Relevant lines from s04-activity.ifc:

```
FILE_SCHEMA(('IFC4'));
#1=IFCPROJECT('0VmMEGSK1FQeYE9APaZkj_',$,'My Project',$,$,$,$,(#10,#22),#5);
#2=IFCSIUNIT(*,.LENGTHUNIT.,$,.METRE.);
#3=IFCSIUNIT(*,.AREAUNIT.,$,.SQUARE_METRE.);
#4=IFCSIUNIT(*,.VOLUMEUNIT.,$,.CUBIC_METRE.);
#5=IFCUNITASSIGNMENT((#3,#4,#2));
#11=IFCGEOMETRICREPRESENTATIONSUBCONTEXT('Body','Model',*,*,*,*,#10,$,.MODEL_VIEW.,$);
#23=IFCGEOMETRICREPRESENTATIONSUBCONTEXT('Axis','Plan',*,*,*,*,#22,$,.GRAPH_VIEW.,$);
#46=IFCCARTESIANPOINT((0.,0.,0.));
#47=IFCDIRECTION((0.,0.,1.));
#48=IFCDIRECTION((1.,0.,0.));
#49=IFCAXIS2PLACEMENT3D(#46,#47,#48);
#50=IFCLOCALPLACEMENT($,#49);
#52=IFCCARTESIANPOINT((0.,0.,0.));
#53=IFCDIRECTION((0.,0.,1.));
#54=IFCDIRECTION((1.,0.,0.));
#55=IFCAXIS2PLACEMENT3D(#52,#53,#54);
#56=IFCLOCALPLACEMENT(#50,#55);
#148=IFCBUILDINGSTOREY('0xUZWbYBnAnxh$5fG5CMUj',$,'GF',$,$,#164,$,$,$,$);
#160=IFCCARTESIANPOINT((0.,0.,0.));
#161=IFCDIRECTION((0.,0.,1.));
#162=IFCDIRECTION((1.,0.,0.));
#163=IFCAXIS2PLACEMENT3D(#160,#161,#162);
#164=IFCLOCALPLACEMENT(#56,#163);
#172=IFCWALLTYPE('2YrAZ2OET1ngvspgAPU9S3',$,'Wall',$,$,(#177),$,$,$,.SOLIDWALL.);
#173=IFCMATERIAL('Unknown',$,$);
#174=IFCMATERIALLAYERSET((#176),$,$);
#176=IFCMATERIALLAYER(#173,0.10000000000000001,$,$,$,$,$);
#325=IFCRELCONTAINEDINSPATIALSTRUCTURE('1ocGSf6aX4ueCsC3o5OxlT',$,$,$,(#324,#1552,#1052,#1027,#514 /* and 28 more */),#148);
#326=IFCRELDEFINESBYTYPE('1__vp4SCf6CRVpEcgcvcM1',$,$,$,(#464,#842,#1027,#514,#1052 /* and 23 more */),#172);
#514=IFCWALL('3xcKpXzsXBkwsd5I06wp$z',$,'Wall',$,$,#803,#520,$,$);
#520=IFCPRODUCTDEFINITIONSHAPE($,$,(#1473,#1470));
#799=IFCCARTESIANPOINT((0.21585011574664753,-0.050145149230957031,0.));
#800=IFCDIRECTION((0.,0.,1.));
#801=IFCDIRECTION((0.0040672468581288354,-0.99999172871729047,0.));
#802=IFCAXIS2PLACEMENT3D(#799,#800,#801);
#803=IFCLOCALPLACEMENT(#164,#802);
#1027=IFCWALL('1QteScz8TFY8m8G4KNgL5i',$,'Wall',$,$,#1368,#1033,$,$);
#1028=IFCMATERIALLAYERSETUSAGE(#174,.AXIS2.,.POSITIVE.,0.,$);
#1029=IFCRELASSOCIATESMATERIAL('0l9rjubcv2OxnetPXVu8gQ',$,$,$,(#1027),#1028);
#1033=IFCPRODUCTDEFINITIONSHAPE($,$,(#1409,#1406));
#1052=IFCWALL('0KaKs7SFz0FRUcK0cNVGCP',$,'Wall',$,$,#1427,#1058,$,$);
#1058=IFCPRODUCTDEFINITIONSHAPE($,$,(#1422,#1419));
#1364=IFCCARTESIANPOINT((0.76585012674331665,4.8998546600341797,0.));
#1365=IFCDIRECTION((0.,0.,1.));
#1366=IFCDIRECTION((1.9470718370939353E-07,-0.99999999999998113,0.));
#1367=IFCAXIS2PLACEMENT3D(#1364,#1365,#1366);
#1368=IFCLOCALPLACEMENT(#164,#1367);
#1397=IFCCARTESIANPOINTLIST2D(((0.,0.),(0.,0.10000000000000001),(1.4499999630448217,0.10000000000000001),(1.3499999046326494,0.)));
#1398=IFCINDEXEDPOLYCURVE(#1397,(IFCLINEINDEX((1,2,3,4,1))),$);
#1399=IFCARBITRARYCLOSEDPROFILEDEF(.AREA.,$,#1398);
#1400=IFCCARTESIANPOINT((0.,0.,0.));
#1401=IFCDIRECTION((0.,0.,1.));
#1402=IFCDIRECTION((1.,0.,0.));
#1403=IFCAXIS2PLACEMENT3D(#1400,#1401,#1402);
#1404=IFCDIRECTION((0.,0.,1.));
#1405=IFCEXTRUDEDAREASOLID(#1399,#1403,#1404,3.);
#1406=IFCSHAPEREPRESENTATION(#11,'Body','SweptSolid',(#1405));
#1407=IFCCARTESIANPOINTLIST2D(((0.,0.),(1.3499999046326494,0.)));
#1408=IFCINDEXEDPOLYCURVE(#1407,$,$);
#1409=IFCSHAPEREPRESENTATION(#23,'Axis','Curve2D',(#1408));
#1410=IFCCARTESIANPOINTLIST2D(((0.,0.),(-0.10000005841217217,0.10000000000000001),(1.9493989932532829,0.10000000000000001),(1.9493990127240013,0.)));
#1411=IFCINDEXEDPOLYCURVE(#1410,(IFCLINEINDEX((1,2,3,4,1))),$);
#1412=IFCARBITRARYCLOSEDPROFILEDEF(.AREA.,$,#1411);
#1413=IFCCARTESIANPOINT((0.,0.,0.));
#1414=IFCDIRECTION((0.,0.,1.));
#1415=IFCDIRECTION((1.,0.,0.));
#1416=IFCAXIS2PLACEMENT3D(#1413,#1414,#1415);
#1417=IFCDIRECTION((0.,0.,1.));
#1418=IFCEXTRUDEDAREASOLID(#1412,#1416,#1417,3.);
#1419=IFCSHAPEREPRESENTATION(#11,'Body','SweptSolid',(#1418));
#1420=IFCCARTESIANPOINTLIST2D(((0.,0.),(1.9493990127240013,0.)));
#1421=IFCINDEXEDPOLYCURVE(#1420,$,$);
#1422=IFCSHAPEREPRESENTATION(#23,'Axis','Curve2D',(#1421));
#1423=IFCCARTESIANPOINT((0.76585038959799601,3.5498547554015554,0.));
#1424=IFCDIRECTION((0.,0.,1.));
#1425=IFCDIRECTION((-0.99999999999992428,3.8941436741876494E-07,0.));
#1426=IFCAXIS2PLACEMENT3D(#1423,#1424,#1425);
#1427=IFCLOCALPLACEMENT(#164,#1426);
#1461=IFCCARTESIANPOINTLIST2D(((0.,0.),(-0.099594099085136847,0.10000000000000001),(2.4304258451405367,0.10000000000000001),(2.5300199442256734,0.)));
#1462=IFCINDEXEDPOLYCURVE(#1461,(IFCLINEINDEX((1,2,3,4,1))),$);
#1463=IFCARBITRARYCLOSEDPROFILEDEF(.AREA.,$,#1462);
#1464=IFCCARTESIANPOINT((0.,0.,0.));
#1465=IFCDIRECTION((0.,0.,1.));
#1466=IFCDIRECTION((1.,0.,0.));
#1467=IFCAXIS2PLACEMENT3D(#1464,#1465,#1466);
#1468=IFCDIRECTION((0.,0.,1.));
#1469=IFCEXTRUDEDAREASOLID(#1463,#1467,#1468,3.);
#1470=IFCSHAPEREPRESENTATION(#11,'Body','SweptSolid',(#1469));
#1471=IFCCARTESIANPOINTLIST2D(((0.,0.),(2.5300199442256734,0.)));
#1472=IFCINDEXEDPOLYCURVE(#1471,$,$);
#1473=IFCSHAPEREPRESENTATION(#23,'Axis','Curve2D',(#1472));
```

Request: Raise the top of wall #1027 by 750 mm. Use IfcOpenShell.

```python
import ifcopenshell
import ifcopenshell.geom
import ifcopenshell.util.representation
import ifcopenshell.util.shape
import ifcopenshell.util.unit

model = ifcopenshell.open("s04-activity.ifc")
unit_scale = ifcopenshell.util.unit.calculate_unit_scale(model)
settings = ifcopenshell.geom.settings()


def volume(element):
    """Net volume in cubic metres, openings subtracted."""
    shape = ifcopenshell.geom.create_shape(settings, element)
    return ifcopenshell.util.shape.get_volume(shape.geometry)


wall = model.by_id(1027)
before = volume(wall)

body = ifcopenshell.util.representation.get_representation(wall, "Model", "Body")
solid = body.Items[0]
old_height = solid.Depth
solid.Depth += 0.75 / unit_scale
after = volume(wall)

print(f"height {old_height:g} -> {solid.Depth:g}, volume {before:.3f} -> {after:.3f} m3")

model.write("s04-activity_v2.ifc")
```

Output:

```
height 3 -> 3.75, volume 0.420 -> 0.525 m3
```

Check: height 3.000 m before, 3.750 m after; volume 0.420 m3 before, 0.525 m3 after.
